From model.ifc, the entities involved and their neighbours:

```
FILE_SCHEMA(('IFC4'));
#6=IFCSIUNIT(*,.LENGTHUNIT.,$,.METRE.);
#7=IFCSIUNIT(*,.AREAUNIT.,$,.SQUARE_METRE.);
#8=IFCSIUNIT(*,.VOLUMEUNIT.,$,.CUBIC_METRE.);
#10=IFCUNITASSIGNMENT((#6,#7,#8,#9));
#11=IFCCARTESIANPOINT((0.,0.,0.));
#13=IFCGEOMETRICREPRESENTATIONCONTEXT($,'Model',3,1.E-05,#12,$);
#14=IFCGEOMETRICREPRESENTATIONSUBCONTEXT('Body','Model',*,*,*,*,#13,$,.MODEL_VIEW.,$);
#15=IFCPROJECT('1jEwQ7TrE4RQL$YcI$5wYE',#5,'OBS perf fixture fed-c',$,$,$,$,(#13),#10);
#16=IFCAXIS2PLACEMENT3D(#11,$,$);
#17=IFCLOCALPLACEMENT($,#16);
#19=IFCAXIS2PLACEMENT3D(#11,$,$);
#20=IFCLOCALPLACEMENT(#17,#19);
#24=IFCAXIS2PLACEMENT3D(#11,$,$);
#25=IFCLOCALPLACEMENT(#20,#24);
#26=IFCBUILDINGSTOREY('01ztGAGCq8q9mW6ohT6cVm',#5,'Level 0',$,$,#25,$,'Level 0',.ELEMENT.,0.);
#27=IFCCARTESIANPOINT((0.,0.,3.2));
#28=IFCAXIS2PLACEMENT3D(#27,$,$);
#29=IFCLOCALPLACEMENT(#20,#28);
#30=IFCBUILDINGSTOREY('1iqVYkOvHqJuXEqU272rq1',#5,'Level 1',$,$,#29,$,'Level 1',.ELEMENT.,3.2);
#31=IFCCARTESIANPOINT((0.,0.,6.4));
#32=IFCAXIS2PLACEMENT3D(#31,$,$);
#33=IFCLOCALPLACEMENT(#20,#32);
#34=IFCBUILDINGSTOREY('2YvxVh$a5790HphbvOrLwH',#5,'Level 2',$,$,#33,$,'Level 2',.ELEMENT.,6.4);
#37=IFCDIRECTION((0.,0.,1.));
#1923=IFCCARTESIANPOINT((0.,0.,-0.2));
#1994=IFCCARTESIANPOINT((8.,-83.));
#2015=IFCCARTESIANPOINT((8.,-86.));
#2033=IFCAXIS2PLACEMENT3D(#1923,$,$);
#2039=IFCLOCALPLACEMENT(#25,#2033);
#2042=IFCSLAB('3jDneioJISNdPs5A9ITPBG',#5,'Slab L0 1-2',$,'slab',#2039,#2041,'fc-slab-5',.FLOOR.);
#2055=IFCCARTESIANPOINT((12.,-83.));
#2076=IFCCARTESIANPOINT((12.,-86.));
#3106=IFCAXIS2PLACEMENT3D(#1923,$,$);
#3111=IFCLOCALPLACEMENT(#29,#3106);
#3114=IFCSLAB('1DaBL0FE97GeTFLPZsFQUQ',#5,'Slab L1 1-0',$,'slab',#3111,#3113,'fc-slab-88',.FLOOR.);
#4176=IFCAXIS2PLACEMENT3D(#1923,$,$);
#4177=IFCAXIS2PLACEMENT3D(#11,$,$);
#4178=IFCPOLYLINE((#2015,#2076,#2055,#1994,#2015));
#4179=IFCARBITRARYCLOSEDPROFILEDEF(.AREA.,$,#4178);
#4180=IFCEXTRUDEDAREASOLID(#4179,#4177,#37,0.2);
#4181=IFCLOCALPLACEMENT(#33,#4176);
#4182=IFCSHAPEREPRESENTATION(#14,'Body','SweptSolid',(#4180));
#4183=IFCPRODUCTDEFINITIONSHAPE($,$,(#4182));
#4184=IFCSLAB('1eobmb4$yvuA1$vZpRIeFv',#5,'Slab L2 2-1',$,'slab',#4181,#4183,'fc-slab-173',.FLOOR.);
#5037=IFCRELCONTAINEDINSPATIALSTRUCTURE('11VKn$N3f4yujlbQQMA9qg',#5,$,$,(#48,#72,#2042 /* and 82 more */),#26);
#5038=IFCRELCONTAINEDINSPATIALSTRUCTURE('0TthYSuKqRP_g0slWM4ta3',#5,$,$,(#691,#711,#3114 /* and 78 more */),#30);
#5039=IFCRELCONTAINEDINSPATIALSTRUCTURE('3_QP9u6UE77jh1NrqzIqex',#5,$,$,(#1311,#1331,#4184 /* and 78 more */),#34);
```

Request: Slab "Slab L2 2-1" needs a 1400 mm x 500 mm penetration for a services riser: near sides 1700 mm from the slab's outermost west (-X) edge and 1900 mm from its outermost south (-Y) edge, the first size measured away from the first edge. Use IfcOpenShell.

```python
import numpy as np
import ifcopenshell
import ifcopenshell.api.feature
import ifcopenshell.api.geometry
import ifcopenshell.api.root
import ifcopenshell.geom
import ifcopenshell.util.placement
import ifcopenshell.util.representation
import ifcopenshell.util.shape
import ifcopenshell.util.unit

model = ifcopenshell.open("model.ifc")
unit_scale = ifcopenshell.util.unit.calculate_unit_scale(model)
settings = ifcopenshell.geom.settings()


def volume(element):
    """Net volume in cubic metres, openings subtracted."""
    shape = ifcopenshell.geom.create_shape(settings, element)
    return ifcopenshell.util.shape.get_volume(shape.geometry)


slab = model.by_guid("1eobmb4$yvuA1$vZpRIeFv")
before = volume(slab)

# Extent in the slab's own axes, in metres. The edges named are its -X and -Y sides.
slab_shape = ifcopenshell.geom.create_shape(settings, slab)
vertices = ifcopenshell.util.shape.get_vertices(slab_shape.geometry)
x_min, y_min, bottom = vertices.min(axis=0)
top = vertices[:, 2].max()

opening = ifcopenshell.api.root.create_entity(model, ifc_class="IfcOpeningElement", name="Services riser opening", predefined_type="OPENING")
context = ifcopenshell.util.representation.get_context(model, "Model", "Body", "MODEL_VIEW")
width, depth = 1.4, 0.5
outline = [(0.0, 0.0), (width, 0.0), (width, depth), (0.0, depth), (0.0, 0.0)]
# Overshoot both faces by 50 mm so the cut is clean.
shape = ifcopenshell.api.geometry.add_slab_representation(
    model, context=context, depth=top - bottom + 0.1, polyline=outline
)
ifcopenshell.api.geometry.assign_representation(model, product=opening, representation=shape)

matrix = ifcopenshell.util.placement.get_local_placement(slab.ObjectPlacement)
matrix[:, 3] = matrix @ np.append(np.array([x_min + 1.7, y_min + 1.9, bottom - 0.05]) / unit_scale, 1.0)
ifcopenshell.api.geometry.edit_object_placement(model, product=opening, matrix=matrix, is_si=False)
ifcopenshell.api.feature.add_feature(model, feature=opening, element=slab)

after = volume(slab)

print(f"slab volume {before:.3f} -> {after:.3f} m3")

model.write("model_updated.ifc")
```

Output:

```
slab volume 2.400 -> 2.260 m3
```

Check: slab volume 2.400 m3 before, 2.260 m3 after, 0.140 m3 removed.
